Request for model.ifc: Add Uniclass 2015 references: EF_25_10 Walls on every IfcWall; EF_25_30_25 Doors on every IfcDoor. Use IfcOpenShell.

First a look at what the model holds.

```python
import ifcopenshell

model = ifcopenshell.open("model.ifc")
print(model.schema)
print("classifications:", [c.Name for c in model.by_type("IfcClassification")])
for ifc_class in ("IfcDoor", "IfcRoof", "IfcStair", "IfcWall", "IfcWindow"):
    print(ifc_class, len(model.by_type(ifc_class)))
```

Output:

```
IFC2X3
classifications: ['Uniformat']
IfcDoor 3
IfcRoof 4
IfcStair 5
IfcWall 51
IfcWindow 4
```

```python
import ifcopenshell
import ifcopenshell.api.classification

model = ifcopenshell.open("model.ifc")

# IFC2X3 requires Source and Edition and has no link from the project to the system.
system = model.create_entity("IfcClassification", Source="NBS", Edition="2015", Name="Uniclass 2015")

codes = {
    "IfcWall": ("EF_25_10", "Walls"),
    "IfcDoor": ("EF_25_30_25", "Doors"),
}
for ifc_class, (code, name) in codes.items():
    products = model.by_type(ifc_class)
    ifcopenshell.api.classification.add_reference(
        model, products=products, classification=system, identification=code, name=name
    )
    print(code, len(products))

model.write("model_updated.ifc")
```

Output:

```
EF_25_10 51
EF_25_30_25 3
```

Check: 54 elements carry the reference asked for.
